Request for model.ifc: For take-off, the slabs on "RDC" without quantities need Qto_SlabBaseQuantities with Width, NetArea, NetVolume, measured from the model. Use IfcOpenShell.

First a look at what the model holds.

```python
import ifcopenshell
import ifcopenshell.util.element
import ifcopenshell.util.unit

model = ifcopenshell.open("model.ifc")
print(model.schema)
for unit_type in ("LENGTHUNIT", "AREAUNIT", "VOLUMEUNIT"):
    print(unit_type, ifcopenshell.util.unit.calculate_unit_scale(model, unit_type))
storey = next(s for s in model.by_type("IfcBuildingStorey") if s.Name == "RDC")
slabs = [e for e in ifcopenshell.util.element.get_decomposition(storey) if e.is_a("IfcSlab")]
for e in sorted(slabs, key=lambda e: e.id()):
    print(e.id(), e.is_a(), e.Name, list(ifcopenshell.util.element.get_psets(e, qtos_only=True)), sep=" | ")
```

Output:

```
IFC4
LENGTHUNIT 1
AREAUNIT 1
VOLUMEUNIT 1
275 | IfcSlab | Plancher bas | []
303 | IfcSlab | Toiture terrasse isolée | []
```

```python
import ifcopenshell
import ifcopenshell.api.pset
import ifcopenshell.geom
import ifcopenshell.util.element
import ifcopenshell.util.shape
import ifcopenshell.util.unit

model = ifcopenshell.open("model.ifc")
unit_scale = ifcopenshell.util.unit.calculate_unit_scale(model)
area_scale = ifcopenshell.util.unit.calculate_unit_scale(model, "AREAUNIT")
volume_scale = ifcopenshell.util.unit.calculate_unit_scale(model, "VOLUMEUNIT")
settings = ifcopenshell.geom.settings()

storey = next(s for s in model.by_type("IfcBuildingStorey") if s.Name == "RDC")
slabs = [e for e in ifcopenshell.util.element.get_decomposition(storey) if e.is_a("IfcSlab")]

for e in sorted(slabs, key=lambda e: e.id()):
    if ifcopenshell.util.element.get_psets(e, qtos_only=True, should_inherit=False):
        continue
    # Geometry comes back in metres, in the element's own axes.
    shape = ifcopenshell.geom.create_shape(settings, e)
    values = {
        "Width": ifcopenshell.util.shape.get_z(shape.geometry) / unit_scale,
        "NetArea": ifcopenshell.util.shape.get_footprint_area(shape.geometry) / area_scale,
        "NetVolume": ifcopenshell.util.shape.get_volume(shape.geometry) / volume_scale,
    }
    qto = ifcopenshell.api.pset.add_qto(model, product=e, name="Qto_SlabBaseQuantities")
    ifcopenshell.api.pset.edit_qto(model, qto=qto, properties=values)
    print(e.id(), {k: round(v, 3) for k, v in values.items()})

model.write("model_rev.ifc")
```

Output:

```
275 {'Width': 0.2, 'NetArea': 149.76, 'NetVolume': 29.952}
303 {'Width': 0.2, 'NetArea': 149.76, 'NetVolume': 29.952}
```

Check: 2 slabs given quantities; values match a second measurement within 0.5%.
